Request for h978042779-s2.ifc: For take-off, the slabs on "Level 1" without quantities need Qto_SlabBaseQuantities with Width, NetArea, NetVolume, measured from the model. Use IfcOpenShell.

First a look at what the model holds.

```python
import ifcopenshell
import ifcopenshell.util.element
import ifcopenshell.util.unit

model = ifcopenshell.open("h978042779-s2.ifc")
print(model.schema)
for unit_type in ("LENGTHUNIT", "AREAUNIT", "VOLUMEUNIT"):
    print(unit_type, ifcopenshell.util.unit.calculate_unit_scale(model, unit_type))
storey = next(s for s in model.by_type("IfcBuildingStorey") if s.Name == "Level 1")
slabs = [e for e in ifcopenshell.util.element.get_decomposition(storey) if e.is_a("IfcSlab")]
for e in sorted(slabs, key=lambda e: e.id()):
    print(e.id(), e.is_a(), e.Name, list(ifcopenshell.util.element.get_psets(e, qtos_only=True)), sep=" | ")
```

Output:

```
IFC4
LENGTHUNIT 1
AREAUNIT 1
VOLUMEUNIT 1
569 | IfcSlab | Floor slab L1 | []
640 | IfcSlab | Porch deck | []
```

```python
import ifcopenshell
import ifcopenshell.api.pset
import ifcopenshell.geom
import ifcopenshell.util.element
import ifcopenshell.util.shape
import ifcopenshell.util.unit

model = ifcopenshell.open("h978042779-s2.ifc")
unit_scale = ifcopenshell.util.unit.calculate_unit_scale(model)
area_scale = ifcopenshell.util.unit.calculate_unit_scale(model, "AREAUNIT")
volume_scale = ifcopenshell.util.unit.calculate_unit_scale(model, "VOLUMEUNIT")
settings = ifcopenshell.geom.settings()

storey = next(s for s in model.by_type("IfcBuildingStorey") if s.Name == "Level 1")
slabs = [e for e in ifcopenshell.util.element.get_decomposition(storey) if e.is_a("IfcSlab")]

for e in sorted(slabs, key=lambda e: e.id()):
    if ifcopenshell.util.element.get_psets(e, qtos_only=True, should_inherit=False):
        continue
    # Geometry comes back in metres, in the element's own axes.
    shape = ifcopenshell.geom.create_shape(settings, e)
    values = {
        "Width": ifcopenshell.util.shape.get_z(shape.geometry) / unit_scale,
        "NetArea": ifcopenshell.util.shape.get_footprint_area(shape.geometry) / area_scale,
        "NetVolume": ifcopenshell.util.shape.get_volume(shape.geometry) / volume_scale,
    }
    qto = ifcopenshell.api.pset.add_qto(model, product=e, name="Qto_SlabBaseQuantities")
    ifcopenshell.api.pset.edit_qto(model, qto=qto, properties=values)
    print(e.id(), {k: round(v, 3) for k, v in values.items()})

model.write("h978042779-s2_rev.ifc")
```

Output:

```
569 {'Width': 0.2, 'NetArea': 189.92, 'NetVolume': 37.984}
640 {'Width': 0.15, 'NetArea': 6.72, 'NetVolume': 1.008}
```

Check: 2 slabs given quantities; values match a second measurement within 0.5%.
